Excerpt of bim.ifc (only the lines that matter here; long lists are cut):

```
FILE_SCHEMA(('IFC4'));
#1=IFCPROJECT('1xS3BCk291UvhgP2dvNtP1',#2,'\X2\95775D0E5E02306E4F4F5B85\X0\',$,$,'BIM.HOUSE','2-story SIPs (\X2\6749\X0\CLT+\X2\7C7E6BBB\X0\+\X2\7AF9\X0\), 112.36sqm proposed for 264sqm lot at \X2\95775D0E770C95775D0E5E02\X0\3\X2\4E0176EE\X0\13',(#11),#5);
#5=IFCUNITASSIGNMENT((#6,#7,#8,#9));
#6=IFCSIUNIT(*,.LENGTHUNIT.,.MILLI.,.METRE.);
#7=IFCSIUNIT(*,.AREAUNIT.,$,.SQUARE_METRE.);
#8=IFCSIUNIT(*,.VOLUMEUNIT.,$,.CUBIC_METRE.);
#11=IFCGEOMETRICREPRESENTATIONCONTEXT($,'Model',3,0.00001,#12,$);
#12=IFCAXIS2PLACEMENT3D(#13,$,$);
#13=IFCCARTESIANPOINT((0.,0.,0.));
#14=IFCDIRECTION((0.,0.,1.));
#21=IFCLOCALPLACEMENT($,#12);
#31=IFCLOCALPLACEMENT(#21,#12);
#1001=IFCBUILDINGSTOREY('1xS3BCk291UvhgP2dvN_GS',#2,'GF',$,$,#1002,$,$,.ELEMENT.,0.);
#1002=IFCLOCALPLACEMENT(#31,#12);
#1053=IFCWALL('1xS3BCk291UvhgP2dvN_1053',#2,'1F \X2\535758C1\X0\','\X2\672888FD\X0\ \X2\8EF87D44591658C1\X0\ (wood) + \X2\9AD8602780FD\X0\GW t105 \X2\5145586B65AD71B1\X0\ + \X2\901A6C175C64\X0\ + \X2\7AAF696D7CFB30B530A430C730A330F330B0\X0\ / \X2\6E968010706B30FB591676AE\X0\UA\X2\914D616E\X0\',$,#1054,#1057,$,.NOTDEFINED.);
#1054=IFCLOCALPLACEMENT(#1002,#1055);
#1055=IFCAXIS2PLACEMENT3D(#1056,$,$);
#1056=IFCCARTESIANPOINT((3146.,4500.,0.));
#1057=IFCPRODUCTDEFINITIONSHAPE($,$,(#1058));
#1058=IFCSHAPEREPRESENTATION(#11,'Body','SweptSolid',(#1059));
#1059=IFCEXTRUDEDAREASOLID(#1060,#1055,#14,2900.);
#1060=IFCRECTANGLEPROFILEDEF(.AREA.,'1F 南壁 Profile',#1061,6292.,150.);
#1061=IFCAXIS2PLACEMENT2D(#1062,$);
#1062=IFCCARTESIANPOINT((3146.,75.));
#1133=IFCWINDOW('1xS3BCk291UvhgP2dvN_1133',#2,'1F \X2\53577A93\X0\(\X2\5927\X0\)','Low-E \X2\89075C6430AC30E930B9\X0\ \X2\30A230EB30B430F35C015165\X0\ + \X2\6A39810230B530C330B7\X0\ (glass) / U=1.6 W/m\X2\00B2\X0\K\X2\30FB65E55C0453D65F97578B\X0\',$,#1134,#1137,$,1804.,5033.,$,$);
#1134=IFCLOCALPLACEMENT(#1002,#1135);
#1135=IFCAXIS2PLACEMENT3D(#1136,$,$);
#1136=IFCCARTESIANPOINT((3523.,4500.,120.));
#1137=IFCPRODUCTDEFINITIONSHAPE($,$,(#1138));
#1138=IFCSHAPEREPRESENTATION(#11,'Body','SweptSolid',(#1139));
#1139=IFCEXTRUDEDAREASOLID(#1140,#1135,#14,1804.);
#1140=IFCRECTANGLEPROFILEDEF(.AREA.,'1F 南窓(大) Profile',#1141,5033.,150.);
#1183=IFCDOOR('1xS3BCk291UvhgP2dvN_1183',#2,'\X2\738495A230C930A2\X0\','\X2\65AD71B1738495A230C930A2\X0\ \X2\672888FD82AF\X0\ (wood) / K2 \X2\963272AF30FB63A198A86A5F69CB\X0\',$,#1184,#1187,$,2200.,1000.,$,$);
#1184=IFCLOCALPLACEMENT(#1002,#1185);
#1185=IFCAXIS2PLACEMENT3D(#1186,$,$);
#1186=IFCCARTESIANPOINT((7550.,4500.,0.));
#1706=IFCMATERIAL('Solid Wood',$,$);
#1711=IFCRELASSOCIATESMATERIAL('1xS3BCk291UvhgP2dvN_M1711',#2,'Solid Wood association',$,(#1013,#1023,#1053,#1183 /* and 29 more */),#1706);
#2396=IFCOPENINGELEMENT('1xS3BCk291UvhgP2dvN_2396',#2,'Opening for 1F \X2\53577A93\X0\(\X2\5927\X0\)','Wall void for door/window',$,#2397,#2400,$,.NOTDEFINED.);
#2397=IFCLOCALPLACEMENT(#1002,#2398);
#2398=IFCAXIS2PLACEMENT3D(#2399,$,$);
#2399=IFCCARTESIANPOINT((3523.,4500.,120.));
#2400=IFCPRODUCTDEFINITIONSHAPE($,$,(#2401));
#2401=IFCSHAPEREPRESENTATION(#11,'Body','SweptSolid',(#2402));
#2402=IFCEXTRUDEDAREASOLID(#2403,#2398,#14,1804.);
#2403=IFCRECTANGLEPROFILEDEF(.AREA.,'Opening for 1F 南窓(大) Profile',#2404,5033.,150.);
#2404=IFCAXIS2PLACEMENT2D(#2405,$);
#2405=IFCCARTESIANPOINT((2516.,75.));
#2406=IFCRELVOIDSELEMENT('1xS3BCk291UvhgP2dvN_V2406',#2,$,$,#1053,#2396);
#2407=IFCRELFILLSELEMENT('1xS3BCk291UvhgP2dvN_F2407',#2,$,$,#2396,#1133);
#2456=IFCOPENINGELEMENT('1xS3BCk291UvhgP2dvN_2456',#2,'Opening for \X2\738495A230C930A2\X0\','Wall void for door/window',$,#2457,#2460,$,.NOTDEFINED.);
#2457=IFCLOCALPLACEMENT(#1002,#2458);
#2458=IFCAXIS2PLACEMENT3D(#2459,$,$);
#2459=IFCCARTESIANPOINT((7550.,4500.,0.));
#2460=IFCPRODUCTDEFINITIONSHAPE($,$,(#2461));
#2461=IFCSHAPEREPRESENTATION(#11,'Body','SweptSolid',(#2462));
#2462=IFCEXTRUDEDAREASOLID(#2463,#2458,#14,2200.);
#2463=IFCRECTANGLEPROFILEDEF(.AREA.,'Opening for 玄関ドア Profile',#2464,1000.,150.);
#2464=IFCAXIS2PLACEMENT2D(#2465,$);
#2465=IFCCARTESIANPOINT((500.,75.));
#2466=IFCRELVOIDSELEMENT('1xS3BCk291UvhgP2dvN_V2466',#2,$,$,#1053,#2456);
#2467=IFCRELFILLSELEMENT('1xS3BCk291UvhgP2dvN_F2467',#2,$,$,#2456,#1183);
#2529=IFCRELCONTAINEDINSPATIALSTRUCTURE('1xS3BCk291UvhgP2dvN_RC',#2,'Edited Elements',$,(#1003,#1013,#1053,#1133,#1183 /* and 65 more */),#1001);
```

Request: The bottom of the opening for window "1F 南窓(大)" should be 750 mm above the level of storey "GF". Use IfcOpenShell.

```python
import numpy as np
import ifcopenshell
import ifcopenshell.api.geometry
import ifcopenshell.geom
import ifcopenshell.util.element
import ifcopenshell.util.placement
import ifcopenshell.util.shape
import ifcopenshell.util.unit

model = ifcopenshell.open("bim.ifc")
unit_scale = ifcopenshell.util.unit.calculate_unit_scale(model)

window = model.by_guid("1xS3BCk291UvhgP2dvN_1133")
opening = window.FillsVoids[0].RelatingOpeningElement
storey = ifcopenshell.util.element.get_container(window, ifc_class="IfcBuildingStorey")
level = ifcopenshell.util.placement.get_local_placement(storey.ObjectPlacement)[2, 3]

# The opening's origin need not be at the sill, so measure its lowest point.
shape = ifcopenshell.geom.create_shape(ifcopenshell.geom.settings(), opening)
bottom = ifcopenshell.util.shape.get_shape_bottom_elevation(shape, shape.geometry) / unit_scale
dz = level + 750.0 - bottom

shift = np.array([0.0, 0.0, dz])
# The window is not placed relative to its opening, so move both.
for product in (opening, window):
    matrix = ifcopenshell.util.placement.get_local_placement(product.ObjectPlacement)
    matrix[:3, 3] += shift
    ifcopenshell.api.geometry.edit_object_placement(model, product=product, matrix=matrix, is_si=False)

print(f"moved by {dz * unit_scale:+.3f} m")

model.write("bim_v2.ifc")
```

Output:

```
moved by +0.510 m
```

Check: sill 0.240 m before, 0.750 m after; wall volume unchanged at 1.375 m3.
